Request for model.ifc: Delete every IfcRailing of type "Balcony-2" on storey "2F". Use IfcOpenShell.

First a look at what the model holds.

```python
import ifcopenshell
import ifcopenshell.util.element

model = ifcopenshell.open("model.ifc")
print(model.schema)
storey = next(s for s in model.by_type("IfcBuildingStorey") if s.Name == "2F")
railings = [e for e in ifcopenshell.util.element.get_decomposition(storey) if e.is_a("IfcRailing")]
seen = {}
for e in railings:
    element_type = ifcopenshell.util.element.get_type(e)
    name = element_type.Name if element_type not in (None, e) else None
    seen[name] = seen.get(name, 0) + 1
for name, count in sorted(seen.items(), key=str):
    print(count, "x", name)
```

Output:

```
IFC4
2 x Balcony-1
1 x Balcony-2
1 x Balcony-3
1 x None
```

```python
import ifcopenshell
import ifcopenshell.api.root
import ifcopenshell.util.element

model = ifcopenshell.open("model.ifc")

storey = next(s for s in model.by_type("IfcBuildingStorey") if s.Name == "2F")
railings = [e for e in ifcopenshell.util.element.get_decomposition(storey) if e.is_a("IfcRailing")]
targets = [e for e in railings if (t := ifcopenshell.util.element.get_type(e)) not in (None, e) and t.Name == "Balcony-2"]

for e in targets:
    ifcopenshell.api.root.remove_product(model, product=e)
print(len(targets), "removed")

model.write("model_rev.ifc")
```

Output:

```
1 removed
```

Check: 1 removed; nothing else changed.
